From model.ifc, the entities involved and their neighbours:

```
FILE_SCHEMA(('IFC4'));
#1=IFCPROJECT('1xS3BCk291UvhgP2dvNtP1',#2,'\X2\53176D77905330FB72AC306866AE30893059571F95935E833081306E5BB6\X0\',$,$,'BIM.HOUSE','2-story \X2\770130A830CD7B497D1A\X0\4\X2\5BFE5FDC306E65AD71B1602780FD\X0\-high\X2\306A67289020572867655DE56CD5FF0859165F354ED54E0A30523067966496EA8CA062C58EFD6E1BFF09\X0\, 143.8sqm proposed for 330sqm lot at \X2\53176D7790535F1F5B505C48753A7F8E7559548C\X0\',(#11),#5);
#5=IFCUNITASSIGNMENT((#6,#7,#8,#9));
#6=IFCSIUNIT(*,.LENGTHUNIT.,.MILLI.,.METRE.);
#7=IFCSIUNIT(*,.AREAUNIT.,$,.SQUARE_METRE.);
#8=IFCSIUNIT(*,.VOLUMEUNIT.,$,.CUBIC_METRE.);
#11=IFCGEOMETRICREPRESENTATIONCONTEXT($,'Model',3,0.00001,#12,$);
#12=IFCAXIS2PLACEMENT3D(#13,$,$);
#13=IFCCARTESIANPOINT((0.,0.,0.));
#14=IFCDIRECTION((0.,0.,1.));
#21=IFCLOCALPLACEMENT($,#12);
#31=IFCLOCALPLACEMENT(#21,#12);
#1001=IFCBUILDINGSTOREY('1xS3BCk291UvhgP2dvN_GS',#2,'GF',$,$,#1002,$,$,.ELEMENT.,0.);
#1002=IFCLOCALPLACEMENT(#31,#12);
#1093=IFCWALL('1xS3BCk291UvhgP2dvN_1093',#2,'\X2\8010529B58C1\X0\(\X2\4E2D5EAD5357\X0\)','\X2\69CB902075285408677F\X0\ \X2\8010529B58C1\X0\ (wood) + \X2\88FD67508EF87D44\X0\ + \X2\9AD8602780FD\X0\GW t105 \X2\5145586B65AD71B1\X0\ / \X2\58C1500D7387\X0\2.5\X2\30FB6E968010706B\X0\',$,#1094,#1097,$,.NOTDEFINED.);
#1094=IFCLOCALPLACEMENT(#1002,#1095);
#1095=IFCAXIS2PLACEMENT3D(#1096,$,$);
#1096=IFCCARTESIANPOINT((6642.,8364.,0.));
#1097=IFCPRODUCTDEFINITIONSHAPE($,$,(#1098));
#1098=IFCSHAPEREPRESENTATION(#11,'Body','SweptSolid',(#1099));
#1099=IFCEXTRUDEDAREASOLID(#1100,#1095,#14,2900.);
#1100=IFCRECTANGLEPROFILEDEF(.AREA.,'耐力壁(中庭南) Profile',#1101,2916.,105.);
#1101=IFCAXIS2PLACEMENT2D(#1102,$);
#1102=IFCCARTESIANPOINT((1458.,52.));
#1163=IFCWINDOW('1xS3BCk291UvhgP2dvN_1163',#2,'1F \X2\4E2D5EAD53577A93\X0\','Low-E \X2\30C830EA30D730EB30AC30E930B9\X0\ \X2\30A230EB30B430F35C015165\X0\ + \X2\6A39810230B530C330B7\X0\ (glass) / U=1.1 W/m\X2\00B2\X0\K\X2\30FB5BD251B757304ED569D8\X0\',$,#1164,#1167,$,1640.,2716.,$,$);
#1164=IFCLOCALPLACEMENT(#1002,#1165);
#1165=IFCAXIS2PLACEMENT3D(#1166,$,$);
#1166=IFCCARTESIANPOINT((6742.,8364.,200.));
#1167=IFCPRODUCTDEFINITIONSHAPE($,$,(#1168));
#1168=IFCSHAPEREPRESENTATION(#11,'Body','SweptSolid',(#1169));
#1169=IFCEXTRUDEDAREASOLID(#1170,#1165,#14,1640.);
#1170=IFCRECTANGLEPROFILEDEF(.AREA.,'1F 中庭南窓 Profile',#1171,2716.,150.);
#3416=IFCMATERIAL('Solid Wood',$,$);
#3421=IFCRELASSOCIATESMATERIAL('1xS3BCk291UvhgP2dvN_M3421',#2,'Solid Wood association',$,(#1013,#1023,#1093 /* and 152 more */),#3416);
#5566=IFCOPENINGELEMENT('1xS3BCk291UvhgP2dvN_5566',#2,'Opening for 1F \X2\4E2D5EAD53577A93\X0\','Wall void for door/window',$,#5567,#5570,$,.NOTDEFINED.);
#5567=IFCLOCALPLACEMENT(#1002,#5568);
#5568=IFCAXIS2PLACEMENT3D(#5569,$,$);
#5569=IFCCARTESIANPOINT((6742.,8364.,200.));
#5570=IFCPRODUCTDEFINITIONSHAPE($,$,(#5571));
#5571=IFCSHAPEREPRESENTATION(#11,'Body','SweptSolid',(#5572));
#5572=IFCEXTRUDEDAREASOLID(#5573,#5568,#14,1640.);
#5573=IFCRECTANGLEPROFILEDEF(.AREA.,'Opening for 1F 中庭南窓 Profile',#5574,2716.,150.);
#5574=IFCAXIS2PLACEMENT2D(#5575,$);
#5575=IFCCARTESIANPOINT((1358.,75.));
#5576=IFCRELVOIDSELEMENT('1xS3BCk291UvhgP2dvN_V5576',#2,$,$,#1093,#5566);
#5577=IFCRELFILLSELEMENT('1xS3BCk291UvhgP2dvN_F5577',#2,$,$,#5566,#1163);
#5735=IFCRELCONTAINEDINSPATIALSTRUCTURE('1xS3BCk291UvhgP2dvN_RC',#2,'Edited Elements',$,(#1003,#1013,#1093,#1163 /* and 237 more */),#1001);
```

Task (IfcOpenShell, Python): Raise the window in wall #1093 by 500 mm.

```python
import numpy as np
import ifcopenshell
import ifcopenshell.api.geometry
import ifcopenshell.util.placement
import ifcopenshell.util.unit

model = ifcopenshell.open("model.ifc")
unit_scale = ifcopenshell.util.unit.calculate_unit_scale(model)

window = model.by_guid("1xS3BCk291UvhgP2dvN_1163")
opening = window.FillsVoids[0].RelatingOpeningElement
dz = 0.5 / unit_scale

shift = np.array([0.0, 0.0, dz])
# The window is not placed relative to its opening, so move both.
for product in (opening, window):
    matrix = ifcopenshell.util.placement.get_local_placement(product.ObjectPlacement)
    matrix[:3, 3] += shift
    ifcopenshell.api.geometry.edit_object_placement(model, product=product, matrix=matrix, is_si=False)

print(f"moved by {dz * unit_scale:+.3f} m")

model.write("model_edited.ifc")
```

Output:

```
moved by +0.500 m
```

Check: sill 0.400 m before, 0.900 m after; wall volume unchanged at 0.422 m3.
